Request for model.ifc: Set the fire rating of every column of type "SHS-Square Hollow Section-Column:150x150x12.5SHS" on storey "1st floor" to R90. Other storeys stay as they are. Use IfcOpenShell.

First a look at what the model holds.

```python
import ifcopenshell
import ifcopenshell.util.element

model = ifcopenshell.open("model.ifc")
print(model.schema)
storey = next(s for s in model.by_type("IfcBuildingStorey") if s.Name == "1st floor")
columns = [e for e in ifcopenshell.util.element.get_decomposition(storey) if e.is_a("IfcColumn")]
seen = {}
for e in columns:
    element_type = ifcopenshell.util.element.get_type(e)
    key = (element_type.Name if element_type != e and element_type else None, ifcopenshell.util.element.get_pset(e, "Pset_ColumnCommon", "FireRating"))
    seen[key] = seen.get(key, 0) + 1
for (name, value), count in sorted(seen.items(), key=str):
    print(count, "x", name, "|", value)
```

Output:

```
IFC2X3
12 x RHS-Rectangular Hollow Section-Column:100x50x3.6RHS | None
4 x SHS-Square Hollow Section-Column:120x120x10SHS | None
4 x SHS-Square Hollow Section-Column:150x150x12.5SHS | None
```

```python
import ifcopenshell
import ifcopenshell.api.pset
import ifcopenshell.util.element

model = ifcopenshell.open("model.ifc")

storey = next(s for s in model.by_type("IfcBuildingStorey") if s.Name == "1st floor")
columns = [e for e in ifcopenshell.util.element.get_decomposition(storey) if e.is_a("IfcColumn")]

count = 0
for e in columns:
    element_type = ifcopenshell.util.element.get_type(e)
    if element_type in (None, e) or element_type.Name != "SHS-Square Hollow Section-Column:150x150x12.5SHS":
        continue
    # add_pset returns the element's existing set when there is one.
    pset = ifcopenshell.api.pset.add_pset(model, product=e, name="Pset_ColumnCommon")
    ifcopenshell.api.pset.edit_pset(model, pset=pset, properties={"FireRating": "R90"})
    count += 1

print(count, "columns updated")

model.write("model_v2.ifc")
```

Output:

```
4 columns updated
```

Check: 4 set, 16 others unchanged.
